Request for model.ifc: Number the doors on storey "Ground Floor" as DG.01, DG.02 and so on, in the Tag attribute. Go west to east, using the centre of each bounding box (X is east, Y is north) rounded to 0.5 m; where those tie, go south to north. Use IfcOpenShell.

First a look at what the model holds.

```python
import ifcopenshell
import ifcopenshell.util.element
import ifcopenshell.util.placement

model = ifcopenshell.open("model.ifc")
print(model.schema)
storey = next(s for s in model.by_type("IfcBuildingStorey") if s.Name == "Ground Floor")
doors = [e for e in ifcopenshell.util.element.get_decomposition(storey) if e.is_a("IfcDoor")]
for e in sorted(doors, key=lambda e: e.id()):
    origin = ifcopenshell.util.placement.get_local_placement(e.ObjectPlacement)[:3, 3]
    print(e.id(), e.Tag, e.Name, origin.round(2) + 0.0, sep=" | ")
```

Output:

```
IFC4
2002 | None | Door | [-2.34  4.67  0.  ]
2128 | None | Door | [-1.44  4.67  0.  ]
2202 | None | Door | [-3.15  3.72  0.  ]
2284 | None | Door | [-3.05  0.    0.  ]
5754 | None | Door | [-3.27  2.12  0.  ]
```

```python
import ifcopenshell
import ifcopenshell.geom
import ifcopenshell.util.element
import ifcopenshell.util.shape

model = ifcopenshell.open("model.ifc")
settings = ifcopenshell.geom.settings()
settings.set("use-world-coords", True)


def centre(element):
    shape = ifcopenshell.geom.create_shape(settings, element)
    return ifcopenshell.util.shape.get_bbox_centroid(shape.geometry)


storey = next(s for s in model.by_type("IfcBuildingStorey") if s.Name == "Ground Floor")
doors = [e for e in ifcopenshell.util.element.get_decomposition(storey) if e.is_a("IfcDoor")]

# Insertion points can sit at a corner or the storey origin, so sort by the geometry (in metres).
centres = {e: centre(e) for e in doors}
doors.sort(key=lambda e: (round(centres[e][0] / 0.5), centres[e][1]))

for i, e in enumerate(doors, start=1):
    number = f"DG.{i:02d}"
    e.Tag = number
    print(e.id(), number)

model.write("model_edited.ifc")
```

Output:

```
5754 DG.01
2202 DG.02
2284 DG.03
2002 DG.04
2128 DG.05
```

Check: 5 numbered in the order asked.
